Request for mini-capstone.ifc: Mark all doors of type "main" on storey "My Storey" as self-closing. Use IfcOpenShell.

First a look at what the model holds.

```python
import ifcopenshell
import ifcopenshell.util.element

model = ifcopenshell.open("mini-capstone.ifc")
print(model.schema)
storey = next(s for s in model.by_type("IfcBuildingStorey") if s.Name == "My Storey")
doors = [e for e in ifcopenshell.util.element.get_decomposition(storey) if e.is_a("IfcDoor")]
seen = {}
for e in doors:
    element_type = ifcopenshell.util.element.get_type(e)
    key = (element_type.Name if element_type != e and element_type else None, ifcopenshell.util.element.get_pset(e, "Pset_DoorCommon", "SelfClosing"))
    seen[key] = seen.get(key, 0) + 1
for (name, value), count in sorted(seen.items(), key=str):
    print(count, "x", name, "|", value)
```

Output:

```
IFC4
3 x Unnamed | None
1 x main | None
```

```python
import ifcopenshell
import ifcopenshell.api.pset
import ifcopenshell.util.element

model = ifcopenshell.open("mini-capstone.ifc")

storey = next(s for s in model.by_type("IfcBuildingStorey") if s.Name == "My Storey")
doors = [e for e in ifcopenshell.util.element.get_decomposition(storey) if e.is_a("IfcDoor")]

count = 0
for e in doors:
    element_type = ifcopenshell.util.element.get_type(e)
    if element_type in (None, e) or element_type.Name != "main":
        continue
    # add_pset returns the element's existing set when there is one.
    pset = ifcopenshell.api.pset.add_pset(model, product=e, name="Pset_DoorCommon")
    ifcopenshell.api.pset.edit_pset(model, pset=pset, properties={"SelfClosing": True})
    count += 1

print(count, "doors updated")

model.write("mini-capstone-out.ifc")
```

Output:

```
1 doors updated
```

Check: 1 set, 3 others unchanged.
